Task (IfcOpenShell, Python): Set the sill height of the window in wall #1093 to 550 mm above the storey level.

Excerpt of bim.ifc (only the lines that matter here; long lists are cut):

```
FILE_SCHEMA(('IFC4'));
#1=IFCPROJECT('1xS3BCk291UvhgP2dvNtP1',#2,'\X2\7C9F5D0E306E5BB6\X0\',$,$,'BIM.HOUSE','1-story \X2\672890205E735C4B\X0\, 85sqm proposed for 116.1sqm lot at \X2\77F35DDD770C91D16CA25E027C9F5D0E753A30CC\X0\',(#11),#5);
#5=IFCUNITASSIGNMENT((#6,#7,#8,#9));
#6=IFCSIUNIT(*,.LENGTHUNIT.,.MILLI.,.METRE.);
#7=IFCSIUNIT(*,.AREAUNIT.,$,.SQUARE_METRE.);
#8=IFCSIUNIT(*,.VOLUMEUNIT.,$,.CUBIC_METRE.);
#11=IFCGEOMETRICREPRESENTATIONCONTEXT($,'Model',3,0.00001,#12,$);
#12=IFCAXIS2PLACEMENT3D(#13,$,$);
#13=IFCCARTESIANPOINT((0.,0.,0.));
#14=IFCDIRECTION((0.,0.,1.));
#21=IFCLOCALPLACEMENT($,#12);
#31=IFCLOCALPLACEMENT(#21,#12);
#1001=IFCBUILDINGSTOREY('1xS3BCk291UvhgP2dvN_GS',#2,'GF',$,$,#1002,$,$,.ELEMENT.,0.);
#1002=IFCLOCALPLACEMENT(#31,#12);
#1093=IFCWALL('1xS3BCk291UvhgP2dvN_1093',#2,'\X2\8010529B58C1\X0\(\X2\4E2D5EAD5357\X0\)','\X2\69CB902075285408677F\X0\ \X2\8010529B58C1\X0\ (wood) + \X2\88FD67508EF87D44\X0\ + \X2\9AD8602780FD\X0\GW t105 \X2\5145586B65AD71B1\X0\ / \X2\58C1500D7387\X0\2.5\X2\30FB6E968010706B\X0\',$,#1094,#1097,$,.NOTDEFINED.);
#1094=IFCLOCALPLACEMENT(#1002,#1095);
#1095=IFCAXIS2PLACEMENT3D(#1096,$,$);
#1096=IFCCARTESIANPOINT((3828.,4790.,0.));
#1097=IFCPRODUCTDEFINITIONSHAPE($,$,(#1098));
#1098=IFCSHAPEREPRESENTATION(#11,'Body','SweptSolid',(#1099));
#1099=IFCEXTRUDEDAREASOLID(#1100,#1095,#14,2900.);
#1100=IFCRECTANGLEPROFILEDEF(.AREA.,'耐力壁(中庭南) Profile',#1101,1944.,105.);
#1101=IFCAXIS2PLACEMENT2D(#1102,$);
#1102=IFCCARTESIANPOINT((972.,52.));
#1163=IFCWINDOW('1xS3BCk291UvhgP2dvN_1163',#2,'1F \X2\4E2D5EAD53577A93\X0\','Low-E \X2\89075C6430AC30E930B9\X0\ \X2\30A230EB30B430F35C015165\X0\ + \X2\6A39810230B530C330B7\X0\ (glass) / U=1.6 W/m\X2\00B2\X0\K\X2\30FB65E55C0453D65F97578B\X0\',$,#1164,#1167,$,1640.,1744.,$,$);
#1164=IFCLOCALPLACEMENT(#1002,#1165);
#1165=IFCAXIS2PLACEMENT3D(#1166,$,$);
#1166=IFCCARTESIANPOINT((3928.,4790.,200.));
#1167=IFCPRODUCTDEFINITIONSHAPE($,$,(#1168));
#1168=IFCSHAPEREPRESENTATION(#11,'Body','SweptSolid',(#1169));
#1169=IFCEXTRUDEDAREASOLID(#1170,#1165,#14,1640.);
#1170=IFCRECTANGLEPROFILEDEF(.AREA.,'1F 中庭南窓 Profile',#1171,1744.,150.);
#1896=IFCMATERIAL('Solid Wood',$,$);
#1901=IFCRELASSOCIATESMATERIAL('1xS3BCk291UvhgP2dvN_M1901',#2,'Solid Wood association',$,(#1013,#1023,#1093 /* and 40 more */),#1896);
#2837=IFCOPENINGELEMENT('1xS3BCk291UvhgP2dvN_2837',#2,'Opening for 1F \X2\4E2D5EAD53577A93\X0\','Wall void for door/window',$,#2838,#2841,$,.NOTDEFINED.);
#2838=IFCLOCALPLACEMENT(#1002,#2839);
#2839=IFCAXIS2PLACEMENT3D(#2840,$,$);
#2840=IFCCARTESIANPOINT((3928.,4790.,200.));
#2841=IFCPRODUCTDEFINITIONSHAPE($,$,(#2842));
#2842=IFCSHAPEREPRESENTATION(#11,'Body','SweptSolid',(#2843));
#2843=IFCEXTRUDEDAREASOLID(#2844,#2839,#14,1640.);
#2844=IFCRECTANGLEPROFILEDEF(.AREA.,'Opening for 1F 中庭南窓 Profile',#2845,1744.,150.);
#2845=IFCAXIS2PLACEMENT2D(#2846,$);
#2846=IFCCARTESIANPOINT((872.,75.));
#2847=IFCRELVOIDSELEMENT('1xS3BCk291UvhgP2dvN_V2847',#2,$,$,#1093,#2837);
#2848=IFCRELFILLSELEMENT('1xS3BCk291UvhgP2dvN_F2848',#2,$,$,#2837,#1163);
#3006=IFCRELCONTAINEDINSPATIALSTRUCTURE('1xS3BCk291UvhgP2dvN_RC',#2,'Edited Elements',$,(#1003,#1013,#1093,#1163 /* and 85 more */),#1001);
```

```python
import numpy as np
import ifcopenshell
import ifcopenshell.api.geometry
import ifcopenshell.geom
import ifcopenshell.util.element
import ifcopenshell.util.placement
import ifcopenshell.util.shape
import ifcopenshell.util.unit

model = ifcopenshell.open("bim.ifc")
unit_scale = ifcopenshell.util.unit.calculate_unit_scale(model)

window = model.by_guid("1xS3BCk291UvhgP2dvN_1163")
opening = window.FillsVoids[0].RelatingOpeningElement
storey = ifcopenshell.util.element.get_container(window, ifc_class="IfcBuildingStorey")
level = ifcopenshell.util.placement.get_local_placement(storey.ObjectPlacement)[2, 3]

# The opening's origin need not be at the sill, so measure its lowest point.
shape = ifcopenshell.geom.create_shape(ifcopenshell.geom.settings(), opening)
bottom = ifcopenshell.util.shape.get_shape_bottom_elevation(shape, shape.geometry) / unit_scale
dz = level + 0.55 / unit_scale - bottom

shift = np.array([0.0, 0.0, dz])
# The window is not placed relative to its opening, so move both.
for product in (opening, window):
    matrix = ifcopenshell.util.placement.get_local_placement(product.ObjectPlacement)
    matrix[:3, 3] += shift
    ifcopenshell.api.geometry.edit_object_placement(model, product=product, matrix=matrix, is_si=False)

print(f"moved by {dz * unit_scale:+.3f} m")

model.write("bim_updated.ifc")
```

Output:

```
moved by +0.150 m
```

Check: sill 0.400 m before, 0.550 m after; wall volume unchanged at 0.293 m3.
